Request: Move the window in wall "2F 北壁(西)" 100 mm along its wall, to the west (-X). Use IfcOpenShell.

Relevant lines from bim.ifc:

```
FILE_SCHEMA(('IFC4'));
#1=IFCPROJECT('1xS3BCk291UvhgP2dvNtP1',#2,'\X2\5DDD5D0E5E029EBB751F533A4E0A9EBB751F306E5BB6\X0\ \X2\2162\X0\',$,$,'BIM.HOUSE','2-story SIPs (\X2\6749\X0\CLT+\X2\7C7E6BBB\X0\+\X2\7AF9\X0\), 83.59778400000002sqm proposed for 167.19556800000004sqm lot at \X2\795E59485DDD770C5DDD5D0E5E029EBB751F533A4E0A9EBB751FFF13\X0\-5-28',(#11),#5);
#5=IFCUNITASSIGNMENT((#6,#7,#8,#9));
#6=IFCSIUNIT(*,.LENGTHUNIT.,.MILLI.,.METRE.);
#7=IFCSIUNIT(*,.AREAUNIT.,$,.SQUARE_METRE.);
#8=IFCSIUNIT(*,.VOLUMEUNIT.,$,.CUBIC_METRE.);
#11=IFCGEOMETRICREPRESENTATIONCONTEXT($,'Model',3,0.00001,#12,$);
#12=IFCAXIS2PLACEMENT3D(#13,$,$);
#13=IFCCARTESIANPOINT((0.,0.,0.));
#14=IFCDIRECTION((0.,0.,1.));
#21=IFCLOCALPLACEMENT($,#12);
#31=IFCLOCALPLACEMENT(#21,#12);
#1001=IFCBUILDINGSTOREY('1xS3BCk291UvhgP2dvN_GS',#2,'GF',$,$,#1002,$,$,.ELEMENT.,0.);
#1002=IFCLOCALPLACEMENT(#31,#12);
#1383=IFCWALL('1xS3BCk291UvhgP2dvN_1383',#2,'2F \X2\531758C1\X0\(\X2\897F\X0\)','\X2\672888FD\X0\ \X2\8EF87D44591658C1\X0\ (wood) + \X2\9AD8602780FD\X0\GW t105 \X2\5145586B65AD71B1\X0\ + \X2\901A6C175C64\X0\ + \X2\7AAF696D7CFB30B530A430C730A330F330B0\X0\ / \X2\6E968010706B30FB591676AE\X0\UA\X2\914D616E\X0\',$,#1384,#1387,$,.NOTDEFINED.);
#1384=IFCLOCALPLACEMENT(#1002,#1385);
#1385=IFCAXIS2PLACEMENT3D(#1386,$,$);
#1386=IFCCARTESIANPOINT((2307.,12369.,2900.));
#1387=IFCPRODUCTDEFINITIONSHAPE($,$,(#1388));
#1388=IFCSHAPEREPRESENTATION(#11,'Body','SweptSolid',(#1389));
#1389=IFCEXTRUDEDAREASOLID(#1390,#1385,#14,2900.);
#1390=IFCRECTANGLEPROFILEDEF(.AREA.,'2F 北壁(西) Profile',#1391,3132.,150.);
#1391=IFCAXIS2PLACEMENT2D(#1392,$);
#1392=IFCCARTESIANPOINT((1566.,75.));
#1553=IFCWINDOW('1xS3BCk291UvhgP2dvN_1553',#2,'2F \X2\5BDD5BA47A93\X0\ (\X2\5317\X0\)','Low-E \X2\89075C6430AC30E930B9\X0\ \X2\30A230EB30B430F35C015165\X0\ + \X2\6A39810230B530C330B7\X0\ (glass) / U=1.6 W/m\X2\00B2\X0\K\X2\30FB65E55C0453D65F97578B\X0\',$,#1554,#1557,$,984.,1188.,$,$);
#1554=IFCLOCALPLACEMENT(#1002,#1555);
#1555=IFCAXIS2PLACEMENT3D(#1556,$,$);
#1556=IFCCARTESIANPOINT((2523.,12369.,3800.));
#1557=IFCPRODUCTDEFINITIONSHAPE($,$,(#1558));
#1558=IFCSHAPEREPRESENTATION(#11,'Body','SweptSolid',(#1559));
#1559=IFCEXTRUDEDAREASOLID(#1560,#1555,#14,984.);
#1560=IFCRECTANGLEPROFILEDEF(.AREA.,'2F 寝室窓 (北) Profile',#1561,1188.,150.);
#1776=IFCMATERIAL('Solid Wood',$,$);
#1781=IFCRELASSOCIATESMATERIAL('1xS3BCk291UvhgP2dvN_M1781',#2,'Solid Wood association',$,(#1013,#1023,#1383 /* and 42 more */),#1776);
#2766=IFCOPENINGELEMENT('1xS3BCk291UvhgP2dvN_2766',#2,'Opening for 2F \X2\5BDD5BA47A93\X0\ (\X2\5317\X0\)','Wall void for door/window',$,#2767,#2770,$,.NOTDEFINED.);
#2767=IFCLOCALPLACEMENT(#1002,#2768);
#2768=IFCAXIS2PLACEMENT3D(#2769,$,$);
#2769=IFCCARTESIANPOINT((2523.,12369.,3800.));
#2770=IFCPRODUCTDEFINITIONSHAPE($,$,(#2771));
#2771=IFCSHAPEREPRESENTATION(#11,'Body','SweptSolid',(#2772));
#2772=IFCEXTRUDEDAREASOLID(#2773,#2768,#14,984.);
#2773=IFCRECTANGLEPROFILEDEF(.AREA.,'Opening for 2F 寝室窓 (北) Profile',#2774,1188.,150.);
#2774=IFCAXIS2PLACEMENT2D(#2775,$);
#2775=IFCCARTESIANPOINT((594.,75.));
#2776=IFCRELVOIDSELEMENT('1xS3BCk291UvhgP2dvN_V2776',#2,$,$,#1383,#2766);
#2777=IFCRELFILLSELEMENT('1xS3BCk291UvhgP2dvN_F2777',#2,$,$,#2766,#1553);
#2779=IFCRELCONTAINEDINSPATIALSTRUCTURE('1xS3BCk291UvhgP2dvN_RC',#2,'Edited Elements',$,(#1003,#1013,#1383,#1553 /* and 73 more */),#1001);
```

```python
import ifcopenshell
import ifcopenshell.api.geometry
import ifcopenshell.util.placement

model = ifcopenshell.open("bim.ifc")

window = model.by_guid("1xS3BCk291UvhgP2dvN_1553")
opening = window.FillsVoids[0].RelatingOpeningElement
wall = opening.VoidsElements[0].RelatingBuildingElement

wall_matrix = ifcopenshell.util.placement.get_local_placement(wall.ObjectPlacement)
shift = wall_matrix[:3, 0] * -100.0
before = ifcopenshell.util.placement.get_local_placement(window.ObjectPlacement)[:3, 3].copy()

# The window is not placed relative to its opening, so move both.
for product in (opening, window):
    matrix = ifcopenshell.util.placement.get_local_placement(product.ObjectPlacement)
    matrix[:3, 3] += shift
    ifcopenshell.api.geometry.edit_object_placement(model, product=product, matrix=matrix, is_si=False)

after = ifcopenshell.util.placement.get_local_placement(window.ObjectPlacement)[:3, 3]
print("window moved by", (after - before).round(3) + 0.0)

model.write("bim_rev.ifc")
```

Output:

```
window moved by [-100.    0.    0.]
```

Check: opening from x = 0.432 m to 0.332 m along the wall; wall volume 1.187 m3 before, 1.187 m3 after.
